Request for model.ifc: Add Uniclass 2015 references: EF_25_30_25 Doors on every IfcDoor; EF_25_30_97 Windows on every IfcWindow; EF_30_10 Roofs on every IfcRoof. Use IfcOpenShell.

First a look at what the model holds.

```python
import ifcopenshell

model = ifcopenshell.open("model.ifc")
print(model.schema)
print("classifications:", [c.Name for c in model.by_type("IfcClassification")])
for ifc_class in ("IfcDoor", "IfcRoof", "IfcStair", "IfcWall", "IfcWindow"):
    print(ifc_class, len(model.by_type(ifc_class)))
```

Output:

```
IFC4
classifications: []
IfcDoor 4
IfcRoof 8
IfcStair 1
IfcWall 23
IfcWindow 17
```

```python
import ifcopenshell
import ifcopenshell.api.classification

model = ifcopenshell.open("model.ifc")

system = ifcopenshell.api.classification.add_classification(model, classification="Uniclass 2015")

codes = {
    "IfcDoor": ("EF_25_30_25", "Doors"),
    "IfcWindow": ("EF_25_30_97", "Windows"),
    "IfcRoof": ("EF_30_10", "Roofs"),
}
for ifc_class, (code, name) in codes.items():
    products = model.by_type(ifc_class)
    ifcopenshell.api.classification.add_reference(
        model, products=products, classification=system, identification=code, name=name
    )
    print(code, len(products))

model.write("model_edited.ifc")
```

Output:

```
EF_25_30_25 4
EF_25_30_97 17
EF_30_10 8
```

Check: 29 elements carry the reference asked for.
